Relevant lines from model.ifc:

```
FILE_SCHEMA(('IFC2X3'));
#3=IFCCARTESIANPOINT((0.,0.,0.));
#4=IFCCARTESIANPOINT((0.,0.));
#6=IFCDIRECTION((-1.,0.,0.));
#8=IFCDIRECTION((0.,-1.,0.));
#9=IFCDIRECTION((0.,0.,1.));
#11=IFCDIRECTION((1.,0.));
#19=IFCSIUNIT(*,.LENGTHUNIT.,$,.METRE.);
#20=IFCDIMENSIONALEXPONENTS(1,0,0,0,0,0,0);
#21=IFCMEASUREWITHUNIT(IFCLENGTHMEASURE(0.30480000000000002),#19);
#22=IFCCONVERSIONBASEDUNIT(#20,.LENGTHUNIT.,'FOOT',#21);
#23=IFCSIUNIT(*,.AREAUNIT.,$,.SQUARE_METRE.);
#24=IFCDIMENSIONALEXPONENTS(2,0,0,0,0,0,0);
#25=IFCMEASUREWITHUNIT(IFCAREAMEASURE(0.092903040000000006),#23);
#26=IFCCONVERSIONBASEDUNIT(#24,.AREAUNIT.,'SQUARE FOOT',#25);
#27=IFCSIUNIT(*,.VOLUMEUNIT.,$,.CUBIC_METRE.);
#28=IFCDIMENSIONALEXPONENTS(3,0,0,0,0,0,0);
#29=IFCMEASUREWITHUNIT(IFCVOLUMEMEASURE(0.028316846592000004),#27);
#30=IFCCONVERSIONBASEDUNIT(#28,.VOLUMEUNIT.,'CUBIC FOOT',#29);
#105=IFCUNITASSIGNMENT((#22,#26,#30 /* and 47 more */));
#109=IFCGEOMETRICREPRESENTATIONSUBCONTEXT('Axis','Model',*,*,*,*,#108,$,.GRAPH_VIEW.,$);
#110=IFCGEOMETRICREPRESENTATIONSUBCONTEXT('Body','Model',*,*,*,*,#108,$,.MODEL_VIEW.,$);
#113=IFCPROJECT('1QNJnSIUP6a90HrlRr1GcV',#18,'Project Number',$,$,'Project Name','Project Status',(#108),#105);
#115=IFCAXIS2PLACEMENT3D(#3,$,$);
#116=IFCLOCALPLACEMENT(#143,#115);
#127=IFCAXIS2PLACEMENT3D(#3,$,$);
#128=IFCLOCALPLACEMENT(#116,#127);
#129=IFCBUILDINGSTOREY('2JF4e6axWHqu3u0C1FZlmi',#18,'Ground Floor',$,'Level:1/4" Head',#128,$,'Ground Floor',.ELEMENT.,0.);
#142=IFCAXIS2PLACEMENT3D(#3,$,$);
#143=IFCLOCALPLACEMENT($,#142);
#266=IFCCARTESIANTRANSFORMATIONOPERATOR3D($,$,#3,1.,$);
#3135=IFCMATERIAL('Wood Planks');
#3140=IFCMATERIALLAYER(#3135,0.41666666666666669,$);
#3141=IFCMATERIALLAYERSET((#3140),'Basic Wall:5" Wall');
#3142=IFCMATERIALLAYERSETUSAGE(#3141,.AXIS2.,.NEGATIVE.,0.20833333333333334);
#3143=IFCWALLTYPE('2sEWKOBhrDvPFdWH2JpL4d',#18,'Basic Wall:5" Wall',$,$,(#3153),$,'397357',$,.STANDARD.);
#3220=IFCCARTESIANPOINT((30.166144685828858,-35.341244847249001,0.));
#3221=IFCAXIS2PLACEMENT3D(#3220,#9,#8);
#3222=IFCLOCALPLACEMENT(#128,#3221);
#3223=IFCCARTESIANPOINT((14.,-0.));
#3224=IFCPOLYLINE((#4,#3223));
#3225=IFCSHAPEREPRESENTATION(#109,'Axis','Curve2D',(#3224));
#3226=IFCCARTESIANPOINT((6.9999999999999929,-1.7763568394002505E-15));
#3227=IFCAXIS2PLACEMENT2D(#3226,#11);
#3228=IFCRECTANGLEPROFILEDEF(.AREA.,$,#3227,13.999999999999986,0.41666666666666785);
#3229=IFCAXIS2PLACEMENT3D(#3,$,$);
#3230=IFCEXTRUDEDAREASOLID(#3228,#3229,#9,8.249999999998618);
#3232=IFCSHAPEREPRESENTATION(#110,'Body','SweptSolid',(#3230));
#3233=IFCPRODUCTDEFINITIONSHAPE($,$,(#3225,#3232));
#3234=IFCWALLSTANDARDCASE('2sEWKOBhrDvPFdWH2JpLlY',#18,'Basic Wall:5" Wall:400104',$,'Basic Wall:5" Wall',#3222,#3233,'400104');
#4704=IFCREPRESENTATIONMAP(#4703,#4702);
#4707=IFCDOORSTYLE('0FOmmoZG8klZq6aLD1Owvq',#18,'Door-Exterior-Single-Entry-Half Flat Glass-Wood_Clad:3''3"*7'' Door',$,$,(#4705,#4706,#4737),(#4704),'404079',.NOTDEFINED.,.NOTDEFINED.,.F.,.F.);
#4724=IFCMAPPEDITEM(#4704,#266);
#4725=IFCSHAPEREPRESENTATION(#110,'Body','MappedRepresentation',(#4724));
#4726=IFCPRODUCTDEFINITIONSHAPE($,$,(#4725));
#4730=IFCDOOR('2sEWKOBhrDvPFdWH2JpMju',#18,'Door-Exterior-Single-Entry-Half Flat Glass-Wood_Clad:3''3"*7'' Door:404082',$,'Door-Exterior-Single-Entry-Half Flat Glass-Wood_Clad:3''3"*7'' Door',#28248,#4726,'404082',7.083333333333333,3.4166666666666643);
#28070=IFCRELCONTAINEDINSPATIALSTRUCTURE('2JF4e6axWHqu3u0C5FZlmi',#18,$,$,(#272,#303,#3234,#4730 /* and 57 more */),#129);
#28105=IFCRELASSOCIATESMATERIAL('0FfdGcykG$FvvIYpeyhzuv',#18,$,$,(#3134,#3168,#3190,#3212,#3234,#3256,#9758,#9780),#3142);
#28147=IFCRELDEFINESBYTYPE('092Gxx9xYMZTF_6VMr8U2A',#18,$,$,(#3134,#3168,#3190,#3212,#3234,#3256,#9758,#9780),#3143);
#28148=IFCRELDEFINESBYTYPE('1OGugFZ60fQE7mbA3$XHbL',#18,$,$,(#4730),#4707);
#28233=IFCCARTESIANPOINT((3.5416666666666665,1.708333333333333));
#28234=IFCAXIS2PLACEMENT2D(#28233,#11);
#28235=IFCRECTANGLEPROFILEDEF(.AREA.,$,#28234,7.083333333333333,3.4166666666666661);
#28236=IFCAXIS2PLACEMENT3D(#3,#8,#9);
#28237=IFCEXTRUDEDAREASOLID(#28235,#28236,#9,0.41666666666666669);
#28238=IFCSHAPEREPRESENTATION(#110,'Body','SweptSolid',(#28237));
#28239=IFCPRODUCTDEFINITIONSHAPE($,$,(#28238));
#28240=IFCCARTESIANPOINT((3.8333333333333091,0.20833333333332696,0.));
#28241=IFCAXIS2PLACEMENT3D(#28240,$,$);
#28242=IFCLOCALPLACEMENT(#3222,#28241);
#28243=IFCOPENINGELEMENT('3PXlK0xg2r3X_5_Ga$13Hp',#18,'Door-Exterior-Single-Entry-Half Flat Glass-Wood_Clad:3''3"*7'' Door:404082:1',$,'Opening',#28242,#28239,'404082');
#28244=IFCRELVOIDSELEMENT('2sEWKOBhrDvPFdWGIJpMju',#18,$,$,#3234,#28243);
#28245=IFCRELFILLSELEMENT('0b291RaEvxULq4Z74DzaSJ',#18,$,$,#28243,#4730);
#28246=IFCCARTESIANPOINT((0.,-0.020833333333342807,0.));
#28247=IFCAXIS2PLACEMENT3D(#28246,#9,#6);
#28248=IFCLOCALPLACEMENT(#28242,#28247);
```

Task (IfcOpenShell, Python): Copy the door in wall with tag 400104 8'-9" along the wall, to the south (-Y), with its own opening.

```python
import ifcopenshell
import ifcopenshell.api.feature
import ifcopenshell.api.geometry
import ifcopenshell.api.root
import ifcopenshell.geom
import ifcopenshell.util.element
import ifcopenshell.util.placement
import ifcopenshell.util.shape
import ifcopenshell.util.unit

model = ifcopenshell.open("model.ifc")
unit_scale = ifcopenshell.util.unit.calculate_unit_scale(model)
settings = ifcopenshell.geom.settings()


def volume(element):
    """Net volume in cubic metres, openings subtracted."""
    shape = ifcopenshell.geom.create_shape(settings, element)
    return ifcopenshell.util.shape.get_volume(shape.geometry)


def reuse_history(source, copy):
    """copy_class also copies each property set's owner history, people and application; keep the originals."""
    for rel in copy.IsDefinedBy:
        if rel.is_a("IfcRelDefinesByProperties") and (history := rel.RelatingPropertyDefinition.OwnerHistory):
            rel.RelatingPropertyDefinition.OwnerHistory = source.OwnerHistory
            ifcopenshell.util.element.remove_deep2(model, history)


door = model.by_guid("2sEWKOBhrDvPFdWH2JpMju")
opening = door.FillsVoids[0].RelatingOpeningElement
wall = opening.VoidsElements[0].RelatingBuildingElement
before = volume(wall)
shift = ifcopenshell.util.placement.get_local_placement(wall.ObjectPlacement)[:3, 0] * 105 * 0.0254 / unit_scale

# copy_class copies the void relationship, type, container and properties, but no geometry.
new_opening = ifcopenshell.api.root.copy_class(model, product=opening)
new_opening.Representation = ifcopenshell.util.element.copy_deep(
    model, opening.Representation, exclude=["IfcGeometricRepresentationContext", "IfcRepresentationMap"]
)
new_opening.Name = 'Door-Exterior-Single-Entry-Half Flat Glass-Wood_Clad:3\'3"*7\' Door'
new_opening.Tag = None
new_door = ifcopenshell.api.root.copy_class(model, product=door)
new_door.Representation = ifcopenshell.util.element.copy_deep(
    model, door.Representation, exclude=["IfcGeometricRepresentationContext", "IfcRepresentationMap"]
)
new_door.Name = 'Door-Exterior-Single-Entry-Half Flat Glass-Wood_Clad:3\'3"*7\' Door'
new_door.Tag = None
reuse_history(door, new_door)
fills = ifcopenshell.api.feature.add_filling(model, opening=new_opening, element=new_door)
fills.OwnerHistory = new_door.OwnerHistory  # required in IFC2X3

for old, new in ((opening, new_opening), (door, new_door)):
    matrix = ifcopenshell.util.placement.get_local_placement(old.ObjectPlacement)
    matrix[:3, 3] += shift
    ifcopenshell.api.geometry.edit_object_placement(model, product=new, matrix=matrix, is_si=False)

after = volume(wall)

print(f"wall volume {before:.3f} -> {after:.3f} m3")

model.write("model_updated.ifc")
```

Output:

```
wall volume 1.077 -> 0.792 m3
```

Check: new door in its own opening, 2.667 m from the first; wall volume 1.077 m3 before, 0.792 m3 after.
